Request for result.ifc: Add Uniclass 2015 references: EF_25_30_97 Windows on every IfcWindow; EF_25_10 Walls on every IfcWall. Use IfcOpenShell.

First a look at what the model holds.

```python
import ifcopenshell

model = ifcopenshell.open("result.ifc")
print(model.schema)
print("classifications:", [c.Name for c in model.by_type("IfcClassification")])
for ifc_class in ("IfcDoor", "IfcRoof", "IfcStair", "IfcWall", "IfcWindow"):
    print(ifc_class, len(model.by_type(ifc_class)))
```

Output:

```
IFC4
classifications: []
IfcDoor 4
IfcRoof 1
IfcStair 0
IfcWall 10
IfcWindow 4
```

```python
import ifcopenshell
import ifcopenshell.api.classification

model = ifcopenshell.open("result.ifc")

system = ifcopenshell.api.classification.add_classification(model, classification="Uniclass 2015")

codes = {
    "IfcWindow": ("EF_25_30_97", "Windows"),
    "IfcWall": ("EF_25_10", "Walls"),
}
for ifc_class, (code, name) in codes.items():
    products = model.by_type(ifc_class)
    ifcopenshell.api.classification.add_reference(
        model, products=products, classification=system, identification=code, name=name
    )
    print(code, len(products))

model.write("result_edited.ifc")
```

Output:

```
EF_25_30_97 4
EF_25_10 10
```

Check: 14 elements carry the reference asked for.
